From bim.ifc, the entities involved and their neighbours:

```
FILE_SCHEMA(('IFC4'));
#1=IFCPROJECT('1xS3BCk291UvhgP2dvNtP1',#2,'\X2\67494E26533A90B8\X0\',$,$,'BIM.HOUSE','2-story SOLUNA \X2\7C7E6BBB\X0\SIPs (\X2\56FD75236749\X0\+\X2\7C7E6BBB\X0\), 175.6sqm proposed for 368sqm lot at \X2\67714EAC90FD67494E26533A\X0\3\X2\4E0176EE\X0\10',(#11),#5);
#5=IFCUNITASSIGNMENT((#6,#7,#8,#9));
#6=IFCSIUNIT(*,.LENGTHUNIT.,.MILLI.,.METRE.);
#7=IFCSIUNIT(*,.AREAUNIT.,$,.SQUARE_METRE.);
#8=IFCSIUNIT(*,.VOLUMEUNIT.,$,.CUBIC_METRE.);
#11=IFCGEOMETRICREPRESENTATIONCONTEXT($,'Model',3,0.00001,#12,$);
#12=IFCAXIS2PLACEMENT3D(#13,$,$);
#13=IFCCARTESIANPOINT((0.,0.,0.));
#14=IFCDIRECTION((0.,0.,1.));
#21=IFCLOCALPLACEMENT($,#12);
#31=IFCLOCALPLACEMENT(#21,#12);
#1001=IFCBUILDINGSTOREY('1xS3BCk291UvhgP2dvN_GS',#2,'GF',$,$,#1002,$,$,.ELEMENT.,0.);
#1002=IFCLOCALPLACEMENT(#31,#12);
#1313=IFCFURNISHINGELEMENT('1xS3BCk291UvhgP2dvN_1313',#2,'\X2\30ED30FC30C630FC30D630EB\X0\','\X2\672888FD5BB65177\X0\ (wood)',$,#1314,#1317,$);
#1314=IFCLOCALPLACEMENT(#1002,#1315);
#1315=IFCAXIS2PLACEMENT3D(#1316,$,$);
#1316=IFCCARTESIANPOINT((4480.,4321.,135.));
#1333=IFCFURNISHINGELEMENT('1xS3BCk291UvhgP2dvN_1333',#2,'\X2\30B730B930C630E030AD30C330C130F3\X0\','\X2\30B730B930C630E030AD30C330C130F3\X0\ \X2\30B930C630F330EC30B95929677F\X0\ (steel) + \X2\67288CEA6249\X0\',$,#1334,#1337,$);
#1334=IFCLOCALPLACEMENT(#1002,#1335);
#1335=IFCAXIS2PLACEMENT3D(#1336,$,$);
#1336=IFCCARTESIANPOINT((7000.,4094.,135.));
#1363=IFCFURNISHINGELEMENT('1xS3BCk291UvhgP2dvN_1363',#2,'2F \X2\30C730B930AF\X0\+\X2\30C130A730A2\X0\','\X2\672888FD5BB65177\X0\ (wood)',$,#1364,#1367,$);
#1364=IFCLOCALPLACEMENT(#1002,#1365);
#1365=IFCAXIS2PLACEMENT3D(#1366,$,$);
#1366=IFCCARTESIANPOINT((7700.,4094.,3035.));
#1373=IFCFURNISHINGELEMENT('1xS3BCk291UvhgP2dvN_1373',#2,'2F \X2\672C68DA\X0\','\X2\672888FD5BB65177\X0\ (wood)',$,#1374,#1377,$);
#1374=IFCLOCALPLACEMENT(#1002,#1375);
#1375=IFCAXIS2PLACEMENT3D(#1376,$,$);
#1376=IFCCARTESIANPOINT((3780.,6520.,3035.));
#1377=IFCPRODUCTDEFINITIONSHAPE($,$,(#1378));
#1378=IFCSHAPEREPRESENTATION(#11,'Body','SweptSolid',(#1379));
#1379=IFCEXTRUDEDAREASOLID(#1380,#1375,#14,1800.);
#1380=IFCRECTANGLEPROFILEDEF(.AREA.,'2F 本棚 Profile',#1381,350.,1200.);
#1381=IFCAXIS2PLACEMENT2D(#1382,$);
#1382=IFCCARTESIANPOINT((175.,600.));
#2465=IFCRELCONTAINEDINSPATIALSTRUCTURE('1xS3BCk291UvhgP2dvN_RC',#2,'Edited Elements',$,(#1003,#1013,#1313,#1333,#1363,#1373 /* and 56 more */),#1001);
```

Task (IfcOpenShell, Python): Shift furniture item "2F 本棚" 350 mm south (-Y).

```python
import ifcopenshell
import ifcopenshell.api.geometry
import ifcopenshell.util.placement

model = ifcopenshell.open("bim.ifc")

item = model.by_id(1373)
matrix = ifcopenshell.util.placement.get_local_placement(item.ObjectPlacement)
matrix[1, 3] -= 350.0
ifcopenshell.api.geometry.edit_object_placement(model, product=item, matrix=matrix, is_si=False)

print(ifcopenshell.util.placement.get_local_placement(item.ObjectPlacement).round(3) + 0.0)

model.write("bim_updated.ifc")
```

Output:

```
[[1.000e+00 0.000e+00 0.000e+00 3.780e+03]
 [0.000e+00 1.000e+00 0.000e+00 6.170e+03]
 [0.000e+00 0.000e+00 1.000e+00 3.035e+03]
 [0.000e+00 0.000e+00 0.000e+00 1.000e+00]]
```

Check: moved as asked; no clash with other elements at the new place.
